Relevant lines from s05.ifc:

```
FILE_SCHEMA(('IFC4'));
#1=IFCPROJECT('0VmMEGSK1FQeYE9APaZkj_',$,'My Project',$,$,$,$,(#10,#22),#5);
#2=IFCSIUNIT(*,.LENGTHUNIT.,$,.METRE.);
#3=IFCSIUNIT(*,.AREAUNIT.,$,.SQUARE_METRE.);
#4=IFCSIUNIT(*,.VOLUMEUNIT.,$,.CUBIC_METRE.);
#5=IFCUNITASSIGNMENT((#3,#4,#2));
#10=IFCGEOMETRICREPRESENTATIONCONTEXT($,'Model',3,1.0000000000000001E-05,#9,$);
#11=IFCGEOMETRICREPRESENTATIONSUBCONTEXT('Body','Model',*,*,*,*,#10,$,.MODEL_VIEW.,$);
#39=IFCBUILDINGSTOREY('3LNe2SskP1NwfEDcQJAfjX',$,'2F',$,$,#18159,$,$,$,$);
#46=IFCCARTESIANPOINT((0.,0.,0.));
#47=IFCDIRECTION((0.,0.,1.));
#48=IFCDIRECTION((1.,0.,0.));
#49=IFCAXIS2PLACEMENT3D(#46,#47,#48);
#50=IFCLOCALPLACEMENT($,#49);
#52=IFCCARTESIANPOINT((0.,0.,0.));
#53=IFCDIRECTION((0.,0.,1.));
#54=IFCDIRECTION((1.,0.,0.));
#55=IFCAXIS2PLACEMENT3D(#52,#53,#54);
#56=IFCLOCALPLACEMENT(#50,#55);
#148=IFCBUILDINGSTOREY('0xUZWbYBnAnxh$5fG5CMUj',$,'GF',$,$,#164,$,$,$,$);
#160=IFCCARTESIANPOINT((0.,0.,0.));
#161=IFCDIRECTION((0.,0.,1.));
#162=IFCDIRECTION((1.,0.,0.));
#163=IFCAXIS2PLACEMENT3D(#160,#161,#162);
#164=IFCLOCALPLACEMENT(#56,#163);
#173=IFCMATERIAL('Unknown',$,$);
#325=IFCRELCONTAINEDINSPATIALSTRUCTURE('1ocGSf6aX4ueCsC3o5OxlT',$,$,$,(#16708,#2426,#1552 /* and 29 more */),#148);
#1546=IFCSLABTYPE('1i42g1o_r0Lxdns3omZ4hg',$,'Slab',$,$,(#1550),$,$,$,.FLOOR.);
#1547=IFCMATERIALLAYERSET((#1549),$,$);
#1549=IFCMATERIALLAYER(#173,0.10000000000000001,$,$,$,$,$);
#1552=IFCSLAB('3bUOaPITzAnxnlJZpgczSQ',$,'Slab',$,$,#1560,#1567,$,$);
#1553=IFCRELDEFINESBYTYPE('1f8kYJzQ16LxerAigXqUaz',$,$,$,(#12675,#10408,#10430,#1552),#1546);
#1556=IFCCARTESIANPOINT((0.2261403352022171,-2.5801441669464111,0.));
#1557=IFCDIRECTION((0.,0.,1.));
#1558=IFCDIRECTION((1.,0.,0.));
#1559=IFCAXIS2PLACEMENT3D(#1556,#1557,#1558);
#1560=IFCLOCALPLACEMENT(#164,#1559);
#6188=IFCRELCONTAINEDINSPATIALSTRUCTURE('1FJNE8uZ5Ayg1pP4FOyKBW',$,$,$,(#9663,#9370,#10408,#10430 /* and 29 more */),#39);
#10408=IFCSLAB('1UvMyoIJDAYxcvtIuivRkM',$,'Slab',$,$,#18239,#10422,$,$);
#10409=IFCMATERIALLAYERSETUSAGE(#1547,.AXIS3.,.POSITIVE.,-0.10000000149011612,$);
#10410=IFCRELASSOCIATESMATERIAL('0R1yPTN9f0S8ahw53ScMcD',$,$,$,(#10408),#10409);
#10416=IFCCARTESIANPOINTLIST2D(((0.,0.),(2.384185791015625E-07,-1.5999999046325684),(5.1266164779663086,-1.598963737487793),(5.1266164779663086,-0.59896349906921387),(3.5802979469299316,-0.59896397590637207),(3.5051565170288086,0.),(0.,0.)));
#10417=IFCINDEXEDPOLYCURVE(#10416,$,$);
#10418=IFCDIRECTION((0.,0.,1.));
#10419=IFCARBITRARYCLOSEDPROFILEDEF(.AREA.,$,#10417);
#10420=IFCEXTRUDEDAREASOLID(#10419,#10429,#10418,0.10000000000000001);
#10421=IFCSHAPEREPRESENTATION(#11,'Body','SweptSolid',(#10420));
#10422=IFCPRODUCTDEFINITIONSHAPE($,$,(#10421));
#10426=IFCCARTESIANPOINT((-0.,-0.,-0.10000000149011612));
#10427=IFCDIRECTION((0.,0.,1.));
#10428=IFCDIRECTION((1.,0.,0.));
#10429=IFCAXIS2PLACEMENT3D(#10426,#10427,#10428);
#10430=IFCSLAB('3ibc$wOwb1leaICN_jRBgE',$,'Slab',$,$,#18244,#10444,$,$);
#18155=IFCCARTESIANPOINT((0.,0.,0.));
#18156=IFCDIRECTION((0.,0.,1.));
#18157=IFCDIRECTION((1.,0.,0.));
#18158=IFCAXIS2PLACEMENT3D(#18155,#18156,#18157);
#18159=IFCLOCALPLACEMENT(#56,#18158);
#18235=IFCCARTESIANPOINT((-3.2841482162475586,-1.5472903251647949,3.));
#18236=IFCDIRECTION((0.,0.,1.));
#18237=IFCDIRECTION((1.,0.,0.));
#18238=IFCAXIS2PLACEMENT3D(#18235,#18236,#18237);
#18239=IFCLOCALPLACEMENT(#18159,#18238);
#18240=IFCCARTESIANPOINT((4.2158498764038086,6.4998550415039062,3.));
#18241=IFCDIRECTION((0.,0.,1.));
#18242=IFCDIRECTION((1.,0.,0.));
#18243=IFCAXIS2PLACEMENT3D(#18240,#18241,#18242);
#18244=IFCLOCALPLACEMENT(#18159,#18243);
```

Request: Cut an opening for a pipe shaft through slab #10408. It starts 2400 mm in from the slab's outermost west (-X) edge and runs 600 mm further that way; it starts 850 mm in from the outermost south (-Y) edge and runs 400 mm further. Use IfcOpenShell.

```python
import numpy as np
import ifcopenshell
import ifcopenshell.api.feature
import ifcopenshell.api.geometry
import ifcopenshell.api.root
import ifcopenshell.geom
import ifcopenshell.util.placement
import ifcopenshell.util.representation
import ifcopenshell.util.shape
import ifcopenshell.util.unit

model = ifcopenshell.open("s05.ifc")
unit_scale = ifcopenshell.util.unit.calculate_unit_scale(model)
settings = ifcopenshell.geom.settings()


def volume(element):
    """Net volume in cubic metres, openings subtracted."""
    shape = ifcopenshell.geom.create_shape(settings, element)
    return ifcopenshell.util.shape.get_volume(shape.geometry)


slab = model.by_guid("1UvMyoIJDAYxcvtIuivRkM")
before = volume(slab)

# Extent in the slab's own axes, in metres. The edges named are its -X and -Y sides.
slab_shape = ifcopenshell.geom.create_shape(settings, slab)
vertices = ifcopenshell.util.shape.get_vertices(slab_shape.geometry)
x_min, y_min, bottom = vertices.min(axis=0)
top = vertices[:, 2].max()

opening = ifcopenshell.api.root.create_entity(model, ifc_class="IfcOpeningElement", name="Pipe shaft opening", predefined_type="OPENING")
context = ifcopenshell.util.representation.get_context(model, "Model", "Body", "MODEL_VIEW")
width, depth = 0.6, 0.4
outline = [(0.0, 0.0), (width, 0.0), (width, depth), (0.0, depth), (0.0, 0.0)]
# Overshoot both faces by 50 mm so the cut is clean.
shape = ifcopenshell.api.geometry.add_slab_representation(
    model, context=context, depth=top - bottom + 0.1, polyline=outline
)
ifcopenshell.api.geometry.assign_representation(model, product=opening, representation=shape)

matrix = ifcopenshell.util.placement.get_local_placement(slab.ObjectPlacement)
matrix[:, 3] = matrix @ np.append(np.array([x_min + 2.4, y_min + 0.85, bottom - 0.05]) / unit_scale, 1.0)
ifcopenshell.api.geometry.edit_object_placement(model, product=opening, matrix=matrix, is_si=False)
ifcopenshell.api.feature.add_feature(model, feature=opening, element=slab)

after = volume(slab)

print(f"slab volume {before:.3f} -> {after:.3f} m3")

model.write("s05_edited.ifc")
```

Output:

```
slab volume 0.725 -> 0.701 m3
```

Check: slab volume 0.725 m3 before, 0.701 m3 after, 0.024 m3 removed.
